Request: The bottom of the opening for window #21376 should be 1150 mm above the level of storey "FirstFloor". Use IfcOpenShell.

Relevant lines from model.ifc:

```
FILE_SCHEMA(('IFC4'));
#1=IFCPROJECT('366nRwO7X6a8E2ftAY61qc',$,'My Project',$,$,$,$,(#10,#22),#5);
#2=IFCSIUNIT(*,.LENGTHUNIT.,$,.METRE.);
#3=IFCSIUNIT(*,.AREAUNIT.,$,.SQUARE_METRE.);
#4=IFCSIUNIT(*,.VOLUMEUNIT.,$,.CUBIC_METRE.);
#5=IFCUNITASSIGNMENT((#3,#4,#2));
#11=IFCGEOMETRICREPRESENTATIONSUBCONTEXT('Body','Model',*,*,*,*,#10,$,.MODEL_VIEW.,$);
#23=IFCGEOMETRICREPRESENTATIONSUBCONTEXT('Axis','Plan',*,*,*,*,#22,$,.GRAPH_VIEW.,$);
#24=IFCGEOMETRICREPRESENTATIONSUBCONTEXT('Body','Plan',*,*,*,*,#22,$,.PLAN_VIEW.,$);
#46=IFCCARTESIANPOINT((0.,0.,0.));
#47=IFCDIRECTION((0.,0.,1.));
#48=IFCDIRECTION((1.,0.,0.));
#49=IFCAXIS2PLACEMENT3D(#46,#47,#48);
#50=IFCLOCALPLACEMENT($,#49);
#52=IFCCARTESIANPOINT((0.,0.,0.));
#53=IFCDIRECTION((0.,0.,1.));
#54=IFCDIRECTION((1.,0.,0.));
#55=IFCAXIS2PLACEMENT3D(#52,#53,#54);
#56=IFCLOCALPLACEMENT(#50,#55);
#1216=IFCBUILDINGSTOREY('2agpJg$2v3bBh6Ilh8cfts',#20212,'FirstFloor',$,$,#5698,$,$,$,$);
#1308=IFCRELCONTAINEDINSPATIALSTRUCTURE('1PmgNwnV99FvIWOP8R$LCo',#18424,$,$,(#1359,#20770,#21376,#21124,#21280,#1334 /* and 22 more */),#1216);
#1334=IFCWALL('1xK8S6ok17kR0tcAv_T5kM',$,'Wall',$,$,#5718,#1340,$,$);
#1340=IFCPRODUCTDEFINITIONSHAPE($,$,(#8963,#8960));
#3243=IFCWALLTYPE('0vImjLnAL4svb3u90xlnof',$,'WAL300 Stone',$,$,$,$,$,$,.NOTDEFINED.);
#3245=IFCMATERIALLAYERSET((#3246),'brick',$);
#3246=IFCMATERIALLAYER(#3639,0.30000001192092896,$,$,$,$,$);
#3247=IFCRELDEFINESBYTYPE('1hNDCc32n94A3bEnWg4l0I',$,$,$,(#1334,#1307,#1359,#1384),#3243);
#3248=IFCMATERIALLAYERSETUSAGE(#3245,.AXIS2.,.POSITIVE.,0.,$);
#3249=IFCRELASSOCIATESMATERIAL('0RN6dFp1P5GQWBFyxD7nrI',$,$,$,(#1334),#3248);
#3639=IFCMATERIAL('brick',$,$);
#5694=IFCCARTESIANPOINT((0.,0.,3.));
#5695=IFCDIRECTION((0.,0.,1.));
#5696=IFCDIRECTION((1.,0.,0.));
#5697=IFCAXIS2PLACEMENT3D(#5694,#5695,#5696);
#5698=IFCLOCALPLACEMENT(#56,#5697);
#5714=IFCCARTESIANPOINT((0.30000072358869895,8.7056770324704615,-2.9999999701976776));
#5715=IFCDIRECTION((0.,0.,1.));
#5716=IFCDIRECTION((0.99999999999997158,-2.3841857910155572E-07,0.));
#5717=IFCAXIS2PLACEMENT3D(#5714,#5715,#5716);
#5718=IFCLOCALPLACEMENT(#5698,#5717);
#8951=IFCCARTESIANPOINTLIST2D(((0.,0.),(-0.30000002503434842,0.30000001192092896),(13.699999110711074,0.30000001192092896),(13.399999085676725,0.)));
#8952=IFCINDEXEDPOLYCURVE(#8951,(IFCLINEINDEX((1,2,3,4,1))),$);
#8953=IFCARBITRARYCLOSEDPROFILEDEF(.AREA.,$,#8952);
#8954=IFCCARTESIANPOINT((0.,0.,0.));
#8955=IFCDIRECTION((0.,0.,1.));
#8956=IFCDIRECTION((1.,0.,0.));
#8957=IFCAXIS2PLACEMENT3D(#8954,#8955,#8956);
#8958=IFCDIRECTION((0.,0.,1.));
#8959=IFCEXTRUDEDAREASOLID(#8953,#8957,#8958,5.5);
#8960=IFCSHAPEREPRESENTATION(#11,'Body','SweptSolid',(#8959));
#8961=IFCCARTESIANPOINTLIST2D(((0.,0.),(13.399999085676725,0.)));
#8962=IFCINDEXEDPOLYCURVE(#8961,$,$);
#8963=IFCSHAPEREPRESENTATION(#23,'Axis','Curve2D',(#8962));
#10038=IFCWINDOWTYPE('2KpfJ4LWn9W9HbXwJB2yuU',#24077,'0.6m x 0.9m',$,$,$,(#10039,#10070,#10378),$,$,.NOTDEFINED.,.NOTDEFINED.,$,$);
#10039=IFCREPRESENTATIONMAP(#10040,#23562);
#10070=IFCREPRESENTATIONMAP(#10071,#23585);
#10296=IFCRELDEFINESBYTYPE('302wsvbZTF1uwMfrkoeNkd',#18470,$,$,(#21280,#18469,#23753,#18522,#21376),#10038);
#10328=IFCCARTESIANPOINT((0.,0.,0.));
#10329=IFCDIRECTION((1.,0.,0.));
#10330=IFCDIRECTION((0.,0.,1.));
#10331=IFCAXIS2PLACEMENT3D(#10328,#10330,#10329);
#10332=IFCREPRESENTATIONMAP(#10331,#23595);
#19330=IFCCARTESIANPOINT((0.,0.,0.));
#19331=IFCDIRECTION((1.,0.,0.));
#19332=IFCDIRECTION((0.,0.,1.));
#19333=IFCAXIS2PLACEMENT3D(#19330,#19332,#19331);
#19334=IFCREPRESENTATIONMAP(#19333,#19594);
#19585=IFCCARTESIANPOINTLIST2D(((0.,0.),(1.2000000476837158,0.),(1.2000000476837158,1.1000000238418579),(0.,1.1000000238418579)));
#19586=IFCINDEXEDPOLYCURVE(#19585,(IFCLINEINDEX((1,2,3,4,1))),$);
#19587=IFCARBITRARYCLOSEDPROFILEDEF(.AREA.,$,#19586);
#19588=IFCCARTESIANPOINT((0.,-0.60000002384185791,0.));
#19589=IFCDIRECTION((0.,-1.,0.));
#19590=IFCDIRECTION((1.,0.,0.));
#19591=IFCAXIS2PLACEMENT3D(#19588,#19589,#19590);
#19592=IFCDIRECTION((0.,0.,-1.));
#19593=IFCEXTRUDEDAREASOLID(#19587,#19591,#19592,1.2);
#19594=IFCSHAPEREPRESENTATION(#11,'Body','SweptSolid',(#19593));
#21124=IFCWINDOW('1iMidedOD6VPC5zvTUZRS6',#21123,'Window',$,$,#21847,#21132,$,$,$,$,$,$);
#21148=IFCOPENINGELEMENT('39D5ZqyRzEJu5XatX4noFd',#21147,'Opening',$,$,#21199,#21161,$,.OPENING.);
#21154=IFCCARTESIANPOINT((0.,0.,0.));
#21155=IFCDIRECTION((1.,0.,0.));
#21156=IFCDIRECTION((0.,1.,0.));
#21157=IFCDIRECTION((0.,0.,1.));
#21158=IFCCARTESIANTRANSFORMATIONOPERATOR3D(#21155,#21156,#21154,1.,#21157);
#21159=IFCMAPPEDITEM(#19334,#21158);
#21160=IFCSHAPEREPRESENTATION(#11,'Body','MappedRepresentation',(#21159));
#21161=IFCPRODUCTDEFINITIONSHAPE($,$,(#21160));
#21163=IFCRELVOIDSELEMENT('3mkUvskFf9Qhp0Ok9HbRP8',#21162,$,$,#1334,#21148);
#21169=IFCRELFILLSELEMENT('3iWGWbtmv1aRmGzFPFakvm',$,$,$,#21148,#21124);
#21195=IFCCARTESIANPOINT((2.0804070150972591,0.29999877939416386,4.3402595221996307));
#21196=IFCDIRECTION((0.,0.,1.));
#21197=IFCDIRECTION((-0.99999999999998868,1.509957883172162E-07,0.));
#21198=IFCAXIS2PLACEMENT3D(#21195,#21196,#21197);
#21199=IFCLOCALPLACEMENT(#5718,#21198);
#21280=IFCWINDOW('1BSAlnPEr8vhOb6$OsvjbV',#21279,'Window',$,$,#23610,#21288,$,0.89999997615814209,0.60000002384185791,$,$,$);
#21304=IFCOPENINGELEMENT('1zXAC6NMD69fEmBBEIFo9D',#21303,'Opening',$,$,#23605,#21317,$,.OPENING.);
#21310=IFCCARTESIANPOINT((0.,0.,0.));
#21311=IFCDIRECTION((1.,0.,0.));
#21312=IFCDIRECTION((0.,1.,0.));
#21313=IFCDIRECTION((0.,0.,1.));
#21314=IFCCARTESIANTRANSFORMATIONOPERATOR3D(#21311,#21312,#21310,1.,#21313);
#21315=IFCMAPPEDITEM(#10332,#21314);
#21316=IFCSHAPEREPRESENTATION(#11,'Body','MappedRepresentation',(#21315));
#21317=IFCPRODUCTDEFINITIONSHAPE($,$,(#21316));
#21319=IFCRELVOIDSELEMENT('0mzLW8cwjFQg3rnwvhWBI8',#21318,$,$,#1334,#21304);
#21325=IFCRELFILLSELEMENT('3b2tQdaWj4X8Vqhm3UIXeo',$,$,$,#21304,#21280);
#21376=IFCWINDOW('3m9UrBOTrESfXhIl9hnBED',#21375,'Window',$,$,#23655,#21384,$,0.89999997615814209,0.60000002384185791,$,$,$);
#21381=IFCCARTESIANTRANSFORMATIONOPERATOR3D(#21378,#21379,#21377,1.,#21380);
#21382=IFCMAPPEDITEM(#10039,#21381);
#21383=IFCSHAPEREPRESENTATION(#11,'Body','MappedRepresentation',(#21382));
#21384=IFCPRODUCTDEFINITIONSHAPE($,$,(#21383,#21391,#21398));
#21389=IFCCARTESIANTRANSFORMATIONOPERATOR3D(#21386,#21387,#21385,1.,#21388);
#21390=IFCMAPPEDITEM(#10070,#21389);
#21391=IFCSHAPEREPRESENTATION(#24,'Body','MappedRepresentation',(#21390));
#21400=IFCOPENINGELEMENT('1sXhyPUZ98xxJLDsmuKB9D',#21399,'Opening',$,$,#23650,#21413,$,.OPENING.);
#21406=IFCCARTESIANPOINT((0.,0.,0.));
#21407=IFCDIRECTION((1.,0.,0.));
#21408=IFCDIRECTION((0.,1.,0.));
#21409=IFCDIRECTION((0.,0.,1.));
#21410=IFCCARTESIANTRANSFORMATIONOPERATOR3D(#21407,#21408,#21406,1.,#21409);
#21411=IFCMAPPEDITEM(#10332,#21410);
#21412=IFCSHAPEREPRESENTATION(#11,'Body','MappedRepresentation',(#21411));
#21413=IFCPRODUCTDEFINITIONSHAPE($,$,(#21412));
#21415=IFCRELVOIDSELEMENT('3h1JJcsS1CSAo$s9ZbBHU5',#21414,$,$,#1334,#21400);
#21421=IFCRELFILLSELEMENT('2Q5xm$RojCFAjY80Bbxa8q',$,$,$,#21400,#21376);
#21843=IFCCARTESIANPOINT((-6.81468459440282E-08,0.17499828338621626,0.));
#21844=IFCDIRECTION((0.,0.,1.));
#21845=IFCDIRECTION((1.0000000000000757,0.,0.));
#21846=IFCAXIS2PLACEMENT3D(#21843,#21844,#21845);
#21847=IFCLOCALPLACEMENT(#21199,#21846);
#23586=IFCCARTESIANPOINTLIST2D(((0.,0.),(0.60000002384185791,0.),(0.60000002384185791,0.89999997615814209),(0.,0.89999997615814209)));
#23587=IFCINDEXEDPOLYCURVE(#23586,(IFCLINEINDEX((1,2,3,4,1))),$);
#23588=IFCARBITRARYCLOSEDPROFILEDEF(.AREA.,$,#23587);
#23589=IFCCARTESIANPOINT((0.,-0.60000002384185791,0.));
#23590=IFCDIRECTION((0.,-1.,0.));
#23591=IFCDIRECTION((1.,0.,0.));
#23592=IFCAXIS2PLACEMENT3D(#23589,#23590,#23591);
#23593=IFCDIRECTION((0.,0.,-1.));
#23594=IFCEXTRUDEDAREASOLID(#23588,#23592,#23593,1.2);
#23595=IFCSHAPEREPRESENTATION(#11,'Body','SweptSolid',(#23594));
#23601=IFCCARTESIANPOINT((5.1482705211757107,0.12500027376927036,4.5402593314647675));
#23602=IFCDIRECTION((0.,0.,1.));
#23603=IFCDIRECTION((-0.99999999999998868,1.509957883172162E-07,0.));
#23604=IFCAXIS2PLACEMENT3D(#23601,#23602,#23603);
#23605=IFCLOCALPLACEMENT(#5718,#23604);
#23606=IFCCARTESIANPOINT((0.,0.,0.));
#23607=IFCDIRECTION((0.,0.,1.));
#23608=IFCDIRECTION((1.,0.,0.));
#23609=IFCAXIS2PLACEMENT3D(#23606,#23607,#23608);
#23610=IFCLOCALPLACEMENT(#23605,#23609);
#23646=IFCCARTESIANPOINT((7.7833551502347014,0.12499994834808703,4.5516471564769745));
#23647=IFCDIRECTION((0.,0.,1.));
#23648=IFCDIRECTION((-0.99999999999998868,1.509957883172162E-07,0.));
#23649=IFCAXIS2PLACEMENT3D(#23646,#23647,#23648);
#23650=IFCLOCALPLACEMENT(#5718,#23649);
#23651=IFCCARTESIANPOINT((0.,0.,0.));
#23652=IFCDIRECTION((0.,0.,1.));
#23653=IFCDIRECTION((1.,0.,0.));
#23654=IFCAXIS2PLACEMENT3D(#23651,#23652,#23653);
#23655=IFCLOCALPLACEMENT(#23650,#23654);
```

```python
import numpy as np
import ifcopenshell
import ifcopenshell.api.geometry
import ifcopenshell.geom
import ifcopenshell.util.element
import ifcopenshell.util.placement
import ifcopenshell.util.shape
import ifcopenshell.util.unit

model = ifcopenshell.open("model.ifc")
unit_scale = ifcopenshell.util.unit.calculate_unit_scale(model)

window = model.by_guid("3m9UrBOTrESfXhIl9hnBED")
opening = window.FillsVoids[0].RelatingOpeningElement
storey = ifcopenshell.util.element.get_container(window, ifc_class="IfcBuildingStorey")
level = ifcopenshell.util.placement.get_local_placement(storey.ObjectPlacement)[2, 3]

# The opening's origin need not be at the sill, so measure its lowest point.
shape = ifcopenshell.geom.create_shape(ifcopenshell.geom.settings(), opening)
bottom = ifcopenshell.util.shape.get_shape_bottom_elevation(shape, shape.geometry) / unit_scale
dz = level + 1.15 / unit_scale - bottom

shift = np.array([0.0, 0.0, dz])
# The window is placed relative to its opening, so it follows when the opening moves.
matrix = ifcopenshell.util.placement.get_local_placement(opening.ObjectPlacement)
matrix[:3, 3] += shift
ifcopenshell.api.geometry.edit_object_placement(
    model, product=opening, matrix=matrix, is_si=False, should_transform_children=True
)

print(f"moved by {dz * unit_scale:+.3f} m")

model.write("model-out.ifc")
```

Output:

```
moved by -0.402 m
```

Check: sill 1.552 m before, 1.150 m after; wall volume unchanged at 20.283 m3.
